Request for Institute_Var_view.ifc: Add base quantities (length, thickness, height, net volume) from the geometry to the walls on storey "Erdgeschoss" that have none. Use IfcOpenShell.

First a look at what the model holds.

```python
import ifcopenshell
import ifcopenshell.util.element
import ifcopenshell.util.unit

model = ifcopenshell.open("Institute_Var_view.ifc")
print(model.schema)
for unit_type in ("LENGTHUNIT", "AREAUNIT", "VOLUMEUNIT"):
    print(unit_type, ifcopenshell.util.unit.calculate_unit_scale(model, unit_type))
storey = next(s for s in model.by_type("IfcBuildingStorey") if s.Name == "Erdgeschoss")
walls = [e for e in ifcopenshell.util.element.get_decomposition(storey) if e.is_a("IfcWall")]
for e in sorted(walls, key=lambda e: e.id()):
    print(e.id(), e.is_a(), e.Name, list(ifcopenshell.util.element.get_psets(e, qtos_only=True)), sep=" | ")
```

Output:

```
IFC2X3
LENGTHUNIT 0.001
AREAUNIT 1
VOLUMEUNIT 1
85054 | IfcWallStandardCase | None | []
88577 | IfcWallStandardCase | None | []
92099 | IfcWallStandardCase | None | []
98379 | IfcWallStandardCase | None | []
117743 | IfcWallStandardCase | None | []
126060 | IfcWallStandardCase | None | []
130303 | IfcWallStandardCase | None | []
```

```python
import ifcopenshell
import ifcopenshell.api.pset
import ifcopenshell.geom
import ifcopenshell.util.element
import ifcopenshell.util.shape
import ifcopenshell.util.unit

model = ifcopenshell.open("Institute_Var_view.ifc")
unit_scale = ifcopenshell.util.unit.calculate_unit_scale(model)
volume_scale = ifcopenshell.util.unit.calculate_unit_scale(model, "VOLUMEUNIT")
settings = ifcopenshell.geom.settings()

storey = next(s for s in model.by_type("IfcBuildingStorey") if s.Name == "Erdgeschoss")
walls = [e for e in ifcopenshell.util.element.get_decomposition(storey) if e.is_a("IfcWall")]

for e in sorted(walls, key=lambda e: e.id()):
    if ifcopenshell.util.element.get_psets(e, qtos_only=True, should_inherit=False):
        continue
    # Geometry comes back in metres, in the element's own axes.
    shape = ifcopenshell.geom.create_shape(settings, e)
    values = {
        "Length": ifcopenshell.util.shape.get_x(shape.geometry) / unit_scale,
        "Width": ifcopenshell.util.shape.get_y(shape.geometry) / unit_scale,
        "Height": ifcopenshell.util.shape.get_z(shape.geometry) / unit_scale,
        "NetVolume": ifcopenshell.util.shape.get_volume(shape.geometry) / volume_scale,
    }
    qto = ifcopenshell.api.pset.add_qto(model, product=e, name="BaseQuantities")
    ifcopenshell.api.pset.edit_qto(model, qto=qto, properties=values)
    print(e.id(), {k: round(v, 3) for k, v in values.items()})

model.write("Institute_Var_view_edited.ifc")
```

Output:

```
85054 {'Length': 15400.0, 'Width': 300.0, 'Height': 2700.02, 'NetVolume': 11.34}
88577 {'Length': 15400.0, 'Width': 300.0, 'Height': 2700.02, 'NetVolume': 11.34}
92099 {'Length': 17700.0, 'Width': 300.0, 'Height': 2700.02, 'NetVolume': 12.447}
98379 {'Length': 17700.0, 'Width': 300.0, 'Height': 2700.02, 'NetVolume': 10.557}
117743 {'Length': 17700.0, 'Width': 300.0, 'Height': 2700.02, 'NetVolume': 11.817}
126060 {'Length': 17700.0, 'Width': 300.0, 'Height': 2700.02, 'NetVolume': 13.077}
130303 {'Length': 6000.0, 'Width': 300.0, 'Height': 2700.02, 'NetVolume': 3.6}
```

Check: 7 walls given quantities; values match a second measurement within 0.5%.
